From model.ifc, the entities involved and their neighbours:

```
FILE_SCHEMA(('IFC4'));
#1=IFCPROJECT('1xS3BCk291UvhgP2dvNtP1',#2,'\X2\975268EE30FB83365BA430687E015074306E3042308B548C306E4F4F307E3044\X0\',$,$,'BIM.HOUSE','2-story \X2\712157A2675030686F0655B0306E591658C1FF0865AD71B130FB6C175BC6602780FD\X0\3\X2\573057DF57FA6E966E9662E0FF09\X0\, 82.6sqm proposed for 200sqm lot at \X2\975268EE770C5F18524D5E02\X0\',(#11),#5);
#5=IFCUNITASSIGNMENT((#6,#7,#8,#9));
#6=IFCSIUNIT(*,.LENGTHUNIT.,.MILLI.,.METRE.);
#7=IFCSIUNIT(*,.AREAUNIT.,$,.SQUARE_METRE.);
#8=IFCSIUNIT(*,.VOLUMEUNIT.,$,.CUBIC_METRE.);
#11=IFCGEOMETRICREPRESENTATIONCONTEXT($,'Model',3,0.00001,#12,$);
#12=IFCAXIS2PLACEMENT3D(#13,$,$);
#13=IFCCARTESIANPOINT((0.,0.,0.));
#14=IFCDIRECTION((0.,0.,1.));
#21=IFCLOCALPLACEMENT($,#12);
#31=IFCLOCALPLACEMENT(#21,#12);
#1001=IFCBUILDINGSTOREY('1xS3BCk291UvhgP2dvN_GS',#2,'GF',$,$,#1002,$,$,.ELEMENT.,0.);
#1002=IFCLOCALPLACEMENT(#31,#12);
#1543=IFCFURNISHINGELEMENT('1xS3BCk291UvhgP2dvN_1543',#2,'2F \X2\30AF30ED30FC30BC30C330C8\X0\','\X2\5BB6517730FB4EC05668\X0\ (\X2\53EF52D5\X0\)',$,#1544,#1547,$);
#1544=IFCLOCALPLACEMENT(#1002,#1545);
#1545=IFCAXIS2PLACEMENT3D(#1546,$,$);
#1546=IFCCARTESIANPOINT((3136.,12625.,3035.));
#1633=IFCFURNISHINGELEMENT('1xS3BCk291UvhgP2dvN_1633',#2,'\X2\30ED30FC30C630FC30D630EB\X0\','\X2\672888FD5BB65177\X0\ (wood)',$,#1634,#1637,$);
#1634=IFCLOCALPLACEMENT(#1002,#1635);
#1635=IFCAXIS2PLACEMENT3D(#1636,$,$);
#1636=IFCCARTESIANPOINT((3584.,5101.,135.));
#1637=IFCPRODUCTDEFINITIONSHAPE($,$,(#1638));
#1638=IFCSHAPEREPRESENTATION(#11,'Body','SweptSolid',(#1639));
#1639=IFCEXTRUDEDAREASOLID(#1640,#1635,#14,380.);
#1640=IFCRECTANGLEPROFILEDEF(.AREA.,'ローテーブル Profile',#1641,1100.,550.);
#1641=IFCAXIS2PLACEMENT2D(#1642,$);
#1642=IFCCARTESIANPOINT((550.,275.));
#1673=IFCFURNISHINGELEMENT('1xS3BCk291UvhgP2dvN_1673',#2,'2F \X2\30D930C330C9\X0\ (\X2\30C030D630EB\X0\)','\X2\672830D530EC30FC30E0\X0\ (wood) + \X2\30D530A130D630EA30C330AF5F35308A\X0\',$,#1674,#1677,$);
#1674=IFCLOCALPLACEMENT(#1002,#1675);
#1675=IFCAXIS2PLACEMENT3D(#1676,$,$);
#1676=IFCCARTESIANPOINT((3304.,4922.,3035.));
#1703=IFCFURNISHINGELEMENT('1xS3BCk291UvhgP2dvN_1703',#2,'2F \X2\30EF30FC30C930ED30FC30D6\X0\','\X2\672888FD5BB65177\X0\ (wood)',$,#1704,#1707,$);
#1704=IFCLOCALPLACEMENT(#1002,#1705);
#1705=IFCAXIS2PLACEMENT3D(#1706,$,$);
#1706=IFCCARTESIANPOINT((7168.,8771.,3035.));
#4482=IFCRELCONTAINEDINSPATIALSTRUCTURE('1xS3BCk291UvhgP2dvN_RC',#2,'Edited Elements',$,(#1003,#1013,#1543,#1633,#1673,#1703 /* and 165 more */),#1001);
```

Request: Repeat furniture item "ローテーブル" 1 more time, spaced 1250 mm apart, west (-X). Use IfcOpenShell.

```python
import numpy as np
import ifcopenshell
import ifcopenshell.api.geometry
import ifcopenshell.api.root
import ifcopenshell.util.element
import ifcopenshell.util.placement
import ifcopenshell.util.unit

model = ifcopenshell.open("model.ifc")
unit_scale = ifcopenshell.util.unit.calculate_unit_scale(model)


def reuse_history(source, copy):
    """copy_class also copies each property set's owner history, people and application; keep the originals."""
    for rel in copy.IsDefinedBy:
        if rel.is_a("IfcRelDefinesByProperties") and (history := rel.RelatingPropertyDefinition.OwnerHistory):
            rel.RelatingPropertyDefinition.OwnerHistory = source.OwnerHistory
            ifcopenshell.util.element.remove_deep2(model, history)


source = model.by_guid("1xS3BCk291UvhgP2dvN_1633")
base = ifcopenshell.util.placement.get_local_placement(source.ObjectPlacement)
step = np.array([-1.0, 0.0, 0.0]) * 1.25 / unit_scale

for i in range(1, 2):
    copy = ifcopenshell.api.root.copy_class(model, product=source)
    copy.Representation = ifcopenshell.util.element.copy_deep(
        model, source.Representation, exclude=["IfcGeometricRepresentationContext", "IfcRepresentationMap"]
    )
    reuse_history(source, copy)
    matrix = base.copy()
    matrix[:3, 3] += i * step
    print("added at", matrix[:3, 3].round(3) + 0.0)
    ifcopenshell.api.geometry.edit_object_placement(model, product=copy, matrix=matrix, is_si=False)

model.write("model_rev.ifc")
```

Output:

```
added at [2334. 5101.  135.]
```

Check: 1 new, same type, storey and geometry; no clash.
